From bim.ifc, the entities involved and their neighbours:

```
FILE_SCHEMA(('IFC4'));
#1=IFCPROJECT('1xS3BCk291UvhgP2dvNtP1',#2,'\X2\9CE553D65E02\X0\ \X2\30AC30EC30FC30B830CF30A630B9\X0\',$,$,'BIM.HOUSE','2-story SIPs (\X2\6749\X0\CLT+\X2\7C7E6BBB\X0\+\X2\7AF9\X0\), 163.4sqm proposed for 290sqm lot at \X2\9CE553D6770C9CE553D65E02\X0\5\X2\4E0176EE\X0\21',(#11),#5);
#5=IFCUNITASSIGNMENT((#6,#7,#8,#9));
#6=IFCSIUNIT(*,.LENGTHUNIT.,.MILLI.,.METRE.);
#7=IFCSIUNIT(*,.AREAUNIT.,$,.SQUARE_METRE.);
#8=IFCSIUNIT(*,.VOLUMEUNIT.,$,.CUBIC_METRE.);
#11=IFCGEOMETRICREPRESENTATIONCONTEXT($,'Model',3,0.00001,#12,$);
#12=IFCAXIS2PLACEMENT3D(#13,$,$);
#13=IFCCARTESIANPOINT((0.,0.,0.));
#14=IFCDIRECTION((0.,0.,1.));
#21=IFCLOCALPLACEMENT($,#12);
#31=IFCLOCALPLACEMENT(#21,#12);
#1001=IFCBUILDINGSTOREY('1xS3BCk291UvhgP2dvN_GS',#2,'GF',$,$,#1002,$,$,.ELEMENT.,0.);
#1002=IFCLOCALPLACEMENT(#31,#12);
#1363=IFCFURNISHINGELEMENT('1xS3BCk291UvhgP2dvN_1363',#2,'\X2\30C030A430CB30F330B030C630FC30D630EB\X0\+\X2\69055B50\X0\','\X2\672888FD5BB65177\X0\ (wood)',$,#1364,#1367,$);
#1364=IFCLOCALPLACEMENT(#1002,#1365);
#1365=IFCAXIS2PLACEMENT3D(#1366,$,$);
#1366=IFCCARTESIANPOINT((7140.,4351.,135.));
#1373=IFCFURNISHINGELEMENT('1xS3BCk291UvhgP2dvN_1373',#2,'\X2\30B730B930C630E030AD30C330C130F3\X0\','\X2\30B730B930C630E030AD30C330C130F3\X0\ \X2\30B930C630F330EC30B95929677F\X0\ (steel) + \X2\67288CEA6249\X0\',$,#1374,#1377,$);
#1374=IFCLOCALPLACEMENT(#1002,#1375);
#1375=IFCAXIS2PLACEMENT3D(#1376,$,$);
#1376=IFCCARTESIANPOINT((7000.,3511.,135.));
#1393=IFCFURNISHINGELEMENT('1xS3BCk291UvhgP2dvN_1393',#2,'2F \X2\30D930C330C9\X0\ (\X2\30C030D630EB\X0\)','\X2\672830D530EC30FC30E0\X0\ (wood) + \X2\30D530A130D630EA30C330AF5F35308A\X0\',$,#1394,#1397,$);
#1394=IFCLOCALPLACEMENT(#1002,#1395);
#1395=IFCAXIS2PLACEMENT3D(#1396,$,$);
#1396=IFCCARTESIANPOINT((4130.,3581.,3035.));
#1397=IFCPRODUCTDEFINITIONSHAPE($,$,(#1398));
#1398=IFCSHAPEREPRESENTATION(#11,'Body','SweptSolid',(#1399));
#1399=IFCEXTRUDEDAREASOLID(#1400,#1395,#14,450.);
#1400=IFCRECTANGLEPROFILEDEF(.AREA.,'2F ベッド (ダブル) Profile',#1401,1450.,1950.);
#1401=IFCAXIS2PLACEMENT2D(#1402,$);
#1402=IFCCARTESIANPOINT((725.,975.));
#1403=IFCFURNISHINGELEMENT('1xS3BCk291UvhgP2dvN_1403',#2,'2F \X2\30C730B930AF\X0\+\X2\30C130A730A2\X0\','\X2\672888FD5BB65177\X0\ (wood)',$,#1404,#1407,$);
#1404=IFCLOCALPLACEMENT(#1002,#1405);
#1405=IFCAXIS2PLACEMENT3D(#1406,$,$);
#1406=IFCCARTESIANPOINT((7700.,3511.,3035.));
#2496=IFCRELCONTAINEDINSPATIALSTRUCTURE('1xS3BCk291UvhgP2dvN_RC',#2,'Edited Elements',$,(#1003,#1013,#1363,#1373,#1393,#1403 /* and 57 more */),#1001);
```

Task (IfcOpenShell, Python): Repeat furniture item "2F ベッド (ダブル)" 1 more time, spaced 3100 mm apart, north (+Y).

```python
import numpy as np
import ifcopenshell
import ifcopenshell.api.geometry
import ifcopenshell.api.root
import ifcopenshell.util.element
import ifcopenshell.util.placement
import ifcopenshell.util.unit

model = ifcopenshell.open("bim.ifc")
unit_scale = ifcopenshell.util.unit.calculate_unit_scale(model)


def reuse_history(source, copy):
    """copy_class also copies each property set's owner history, people and application; keep the originals."""
    for rel in copy.IsDefinedBy:
        if rel.is_a("IfcRelDefinesByProperties") and (history := rel.RelatingPropertyDefinition.OwnerHistory):
            rel.RelatingPropertyDefinition.OwnerHistory = source.OwnerHistory
            ifcopenshell.util.element.remove_deep2(model, history)


source = model.by_guid("1xS3BCk291UvhgP2dvN_1393")
base = ifcopenshell.util.placement.get_local_placement(source.ObjectPlacement)
step = np.array([0.0, 1.0, 0.0]) * 3.1 / unit_scale

for i in range(1, 2):
    copy = ifcopenshell.api.root.copy_class(model, product=source)
    copy.Representation = ifcopenshell.util.element.copy_deep(
        model, source.Representation, exclude=["IfcGeometricRepresentationContext", "IfcRepresentationMap"]
    )
    reuse_history(source, copy)
    matrix = base.copy()
    matrix[:3, 3] += i * step
    print("added at", matrix[:3, 3].round(3) + 0.0)
    ifcopenshell.api.geometry.edit_object_placement(model, product=copy, matrix=matrix, is_si=False)

model.write("bim_updated.ifc")
```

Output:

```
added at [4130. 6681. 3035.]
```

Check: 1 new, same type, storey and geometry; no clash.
